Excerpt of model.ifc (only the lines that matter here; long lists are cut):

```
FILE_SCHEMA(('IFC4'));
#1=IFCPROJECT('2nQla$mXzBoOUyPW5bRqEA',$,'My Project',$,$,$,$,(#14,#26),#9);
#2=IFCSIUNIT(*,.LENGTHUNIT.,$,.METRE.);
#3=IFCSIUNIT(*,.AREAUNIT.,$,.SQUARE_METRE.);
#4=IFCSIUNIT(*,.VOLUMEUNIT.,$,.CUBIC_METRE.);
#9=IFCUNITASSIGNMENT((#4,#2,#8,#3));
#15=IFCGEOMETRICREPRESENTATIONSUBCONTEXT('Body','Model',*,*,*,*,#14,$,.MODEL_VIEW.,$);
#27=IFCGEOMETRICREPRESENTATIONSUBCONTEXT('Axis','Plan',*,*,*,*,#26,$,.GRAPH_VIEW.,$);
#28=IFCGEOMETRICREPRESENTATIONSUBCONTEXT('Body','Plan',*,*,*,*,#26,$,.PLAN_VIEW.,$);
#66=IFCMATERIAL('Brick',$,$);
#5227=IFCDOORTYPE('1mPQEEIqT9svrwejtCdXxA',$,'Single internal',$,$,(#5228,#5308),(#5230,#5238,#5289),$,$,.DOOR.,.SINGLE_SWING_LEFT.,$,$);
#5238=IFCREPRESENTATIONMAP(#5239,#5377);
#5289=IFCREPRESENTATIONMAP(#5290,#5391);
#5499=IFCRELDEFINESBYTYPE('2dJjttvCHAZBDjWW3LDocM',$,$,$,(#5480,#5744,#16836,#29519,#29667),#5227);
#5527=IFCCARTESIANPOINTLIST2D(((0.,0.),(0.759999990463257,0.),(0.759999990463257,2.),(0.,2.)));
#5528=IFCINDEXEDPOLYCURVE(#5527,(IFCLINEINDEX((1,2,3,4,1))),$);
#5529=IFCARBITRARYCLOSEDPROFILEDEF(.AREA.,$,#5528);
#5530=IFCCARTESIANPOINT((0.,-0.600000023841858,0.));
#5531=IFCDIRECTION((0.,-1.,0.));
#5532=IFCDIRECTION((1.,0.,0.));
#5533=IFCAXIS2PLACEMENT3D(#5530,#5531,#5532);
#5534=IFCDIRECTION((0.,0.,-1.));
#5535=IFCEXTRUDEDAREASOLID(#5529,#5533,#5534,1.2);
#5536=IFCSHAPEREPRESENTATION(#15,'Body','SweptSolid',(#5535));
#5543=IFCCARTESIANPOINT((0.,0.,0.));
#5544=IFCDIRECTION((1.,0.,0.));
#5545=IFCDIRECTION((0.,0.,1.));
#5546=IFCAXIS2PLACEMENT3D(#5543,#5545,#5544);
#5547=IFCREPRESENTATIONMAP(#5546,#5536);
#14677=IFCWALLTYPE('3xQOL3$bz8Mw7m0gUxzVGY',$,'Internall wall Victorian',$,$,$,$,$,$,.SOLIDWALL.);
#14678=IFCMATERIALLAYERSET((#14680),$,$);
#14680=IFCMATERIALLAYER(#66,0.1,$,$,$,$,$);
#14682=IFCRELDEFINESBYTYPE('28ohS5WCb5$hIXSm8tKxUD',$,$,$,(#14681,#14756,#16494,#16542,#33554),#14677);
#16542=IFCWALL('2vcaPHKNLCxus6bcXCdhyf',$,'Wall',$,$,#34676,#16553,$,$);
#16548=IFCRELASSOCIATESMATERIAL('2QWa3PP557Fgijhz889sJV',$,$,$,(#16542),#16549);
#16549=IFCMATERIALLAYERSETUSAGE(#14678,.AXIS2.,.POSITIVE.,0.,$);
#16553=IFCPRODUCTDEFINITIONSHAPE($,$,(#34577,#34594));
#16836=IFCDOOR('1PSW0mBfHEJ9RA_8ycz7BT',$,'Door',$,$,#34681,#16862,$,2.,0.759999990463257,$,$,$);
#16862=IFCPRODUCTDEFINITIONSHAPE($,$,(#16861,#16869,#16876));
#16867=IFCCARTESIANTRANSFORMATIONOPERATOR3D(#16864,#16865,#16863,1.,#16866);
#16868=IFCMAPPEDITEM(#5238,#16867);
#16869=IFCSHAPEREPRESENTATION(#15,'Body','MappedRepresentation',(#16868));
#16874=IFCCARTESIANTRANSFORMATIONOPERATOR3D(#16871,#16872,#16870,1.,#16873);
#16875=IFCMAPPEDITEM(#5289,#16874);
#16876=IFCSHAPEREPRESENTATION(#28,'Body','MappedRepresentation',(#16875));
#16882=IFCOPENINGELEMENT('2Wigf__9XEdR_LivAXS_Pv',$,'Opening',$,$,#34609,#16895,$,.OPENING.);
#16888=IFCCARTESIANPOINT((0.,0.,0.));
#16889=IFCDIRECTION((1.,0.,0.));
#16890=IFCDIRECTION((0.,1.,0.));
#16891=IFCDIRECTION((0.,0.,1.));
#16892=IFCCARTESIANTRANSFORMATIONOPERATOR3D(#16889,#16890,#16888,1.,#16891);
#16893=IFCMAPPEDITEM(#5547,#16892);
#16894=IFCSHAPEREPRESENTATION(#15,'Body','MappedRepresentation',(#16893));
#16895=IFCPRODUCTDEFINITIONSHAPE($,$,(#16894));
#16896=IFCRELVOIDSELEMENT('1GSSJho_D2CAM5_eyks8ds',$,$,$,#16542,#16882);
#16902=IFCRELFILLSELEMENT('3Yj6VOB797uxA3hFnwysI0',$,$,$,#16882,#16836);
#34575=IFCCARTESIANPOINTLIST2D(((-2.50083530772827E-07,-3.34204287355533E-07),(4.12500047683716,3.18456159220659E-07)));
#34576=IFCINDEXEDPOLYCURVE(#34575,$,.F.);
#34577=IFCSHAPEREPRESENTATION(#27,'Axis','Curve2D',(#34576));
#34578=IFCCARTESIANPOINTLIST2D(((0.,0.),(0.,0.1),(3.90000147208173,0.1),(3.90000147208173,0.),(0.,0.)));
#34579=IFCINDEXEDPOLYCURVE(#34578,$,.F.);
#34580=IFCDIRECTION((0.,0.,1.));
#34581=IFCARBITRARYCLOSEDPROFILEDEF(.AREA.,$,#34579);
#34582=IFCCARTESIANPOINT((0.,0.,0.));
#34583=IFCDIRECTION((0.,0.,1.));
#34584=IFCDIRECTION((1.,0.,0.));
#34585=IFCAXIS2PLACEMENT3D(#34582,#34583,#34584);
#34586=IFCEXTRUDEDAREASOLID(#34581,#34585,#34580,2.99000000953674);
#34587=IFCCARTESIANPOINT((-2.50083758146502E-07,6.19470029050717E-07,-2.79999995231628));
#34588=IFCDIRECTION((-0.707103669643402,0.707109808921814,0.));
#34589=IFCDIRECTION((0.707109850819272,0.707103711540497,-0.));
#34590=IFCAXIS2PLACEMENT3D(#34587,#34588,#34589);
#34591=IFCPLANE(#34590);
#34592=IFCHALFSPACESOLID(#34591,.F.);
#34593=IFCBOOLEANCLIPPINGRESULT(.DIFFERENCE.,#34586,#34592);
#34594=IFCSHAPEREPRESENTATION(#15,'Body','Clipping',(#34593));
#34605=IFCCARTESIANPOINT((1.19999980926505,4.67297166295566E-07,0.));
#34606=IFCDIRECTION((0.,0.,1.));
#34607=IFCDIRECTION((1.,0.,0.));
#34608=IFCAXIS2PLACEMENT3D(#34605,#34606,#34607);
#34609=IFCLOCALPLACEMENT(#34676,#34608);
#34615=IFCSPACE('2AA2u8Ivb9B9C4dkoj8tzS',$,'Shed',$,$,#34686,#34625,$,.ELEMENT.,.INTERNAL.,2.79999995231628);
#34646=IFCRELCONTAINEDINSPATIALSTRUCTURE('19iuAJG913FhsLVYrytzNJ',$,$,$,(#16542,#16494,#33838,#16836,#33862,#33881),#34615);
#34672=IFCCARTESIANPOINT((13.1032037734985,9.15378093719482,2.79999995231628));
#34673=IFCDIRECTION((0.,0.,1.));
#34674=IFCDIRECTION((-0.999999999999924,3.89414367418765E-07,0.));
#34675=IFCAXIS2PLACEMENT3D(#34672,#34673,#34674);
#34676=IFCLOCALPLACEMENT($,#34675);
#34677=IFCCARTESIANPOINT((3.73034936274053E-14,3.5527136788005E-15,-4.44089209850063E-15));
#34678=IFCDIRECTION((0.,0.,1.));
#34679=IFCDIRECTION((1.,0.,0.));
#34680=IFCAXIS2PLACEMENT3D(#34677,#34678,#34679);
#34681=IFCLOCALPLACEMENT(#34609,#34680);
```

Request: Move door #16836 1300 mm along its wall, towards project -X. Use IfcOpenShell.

```python
import ifcopenshell
import ifcopenshell.api.geometry
import ifcopenshell.util.placement
import ifcopenshell.util.unit

model = ifcopenshell.open("model.ifc")
unit_scale = ifcopenshell.util.unit.calculate_unit_scale(model)

door = model.by_guid("1PSW0mBfHEJ9RA_8ycz7BT")
opening = door.FillsVoids[0].RelatingOpeningElement
wall = opening.VoidsElements[0].RelatingBuildingElement

wall_matrix = ifcopenshell.util.placement.get_local_placement(wall.ObjectPlacement)
shift = wall_matrix[:3, 0] * 1.3 / unit_scale
before = ifcopenshell.util.placement.get_local_placement(door.ObjectPlacement)[:3, 3].copy()

# The door is placed relative to its opening, so it follows when the opening moves.
matrix = ifcopenshell.util.placement.get_local_placement(opening.ObjectPlacement)
matrix[:3, 3] += shift
ifcopenshell.api.geometry.edit_object_placement(
    model, product=opening, matrix=matrix, is_si=False, should_transform_children=True
)

after = ifcopenshell.util.placement.get_local_placement(door.ObjectPlacement)[:3, 3]
print("door moved by", (after - before).round(3) + 0.0)

model.write("model-out.ifc")
```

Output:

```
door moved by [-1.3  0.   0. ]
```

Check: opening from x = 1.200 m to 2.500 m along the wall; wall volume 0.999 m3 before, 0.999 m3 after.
